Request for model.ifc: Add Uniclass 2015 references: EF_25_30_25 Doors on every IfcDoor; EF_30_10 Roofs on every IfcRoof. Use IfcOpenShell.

First a look at what the model holds.

```python
import ifcopenshell

model = ifcopenshell.open("model.ifc")
print(model.schema)
print("classifications:", [c.Name for c in model.by_type("IfcClassification")])
for ifc_class in ("IfcDoor", "IfcRoof", "IfcStair", "IfcWall", "IfcWindow"):
    print(ifc_class, len(model.by_type(ifc_class)))
```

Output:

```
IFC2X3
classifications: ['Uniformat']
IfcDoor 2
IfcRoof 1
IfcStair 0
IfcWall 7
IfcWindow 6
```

```python
import ifcopenshell
import ifcopenshell.api.classification

model = ifcopenshell.open("model.ifc")

# IFC2X3 requires Source and Edition and has no link from the project to the system.
system = model.create_entity("IfcClassification", Source="NBS", Edition="2015", Name="Uniclass 2015")

codes = {
    "IfcDoor": ("EF_25_30_25", "Doors"),
    "IfcRoof": ("EF_30_10", "Roofs"),
}
for ifc_class, (code, name) in codes.items():
    products = model.by_type(ifc_class)
    ifcopenshell.api.classification.add_reference(
        model, products=products, classification=system, identification=code, name=name
    )
    print(code, len(products))

model.write("model_rev.ifc")
```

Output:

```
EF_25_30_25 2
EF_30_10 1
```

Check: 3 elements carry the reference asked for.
